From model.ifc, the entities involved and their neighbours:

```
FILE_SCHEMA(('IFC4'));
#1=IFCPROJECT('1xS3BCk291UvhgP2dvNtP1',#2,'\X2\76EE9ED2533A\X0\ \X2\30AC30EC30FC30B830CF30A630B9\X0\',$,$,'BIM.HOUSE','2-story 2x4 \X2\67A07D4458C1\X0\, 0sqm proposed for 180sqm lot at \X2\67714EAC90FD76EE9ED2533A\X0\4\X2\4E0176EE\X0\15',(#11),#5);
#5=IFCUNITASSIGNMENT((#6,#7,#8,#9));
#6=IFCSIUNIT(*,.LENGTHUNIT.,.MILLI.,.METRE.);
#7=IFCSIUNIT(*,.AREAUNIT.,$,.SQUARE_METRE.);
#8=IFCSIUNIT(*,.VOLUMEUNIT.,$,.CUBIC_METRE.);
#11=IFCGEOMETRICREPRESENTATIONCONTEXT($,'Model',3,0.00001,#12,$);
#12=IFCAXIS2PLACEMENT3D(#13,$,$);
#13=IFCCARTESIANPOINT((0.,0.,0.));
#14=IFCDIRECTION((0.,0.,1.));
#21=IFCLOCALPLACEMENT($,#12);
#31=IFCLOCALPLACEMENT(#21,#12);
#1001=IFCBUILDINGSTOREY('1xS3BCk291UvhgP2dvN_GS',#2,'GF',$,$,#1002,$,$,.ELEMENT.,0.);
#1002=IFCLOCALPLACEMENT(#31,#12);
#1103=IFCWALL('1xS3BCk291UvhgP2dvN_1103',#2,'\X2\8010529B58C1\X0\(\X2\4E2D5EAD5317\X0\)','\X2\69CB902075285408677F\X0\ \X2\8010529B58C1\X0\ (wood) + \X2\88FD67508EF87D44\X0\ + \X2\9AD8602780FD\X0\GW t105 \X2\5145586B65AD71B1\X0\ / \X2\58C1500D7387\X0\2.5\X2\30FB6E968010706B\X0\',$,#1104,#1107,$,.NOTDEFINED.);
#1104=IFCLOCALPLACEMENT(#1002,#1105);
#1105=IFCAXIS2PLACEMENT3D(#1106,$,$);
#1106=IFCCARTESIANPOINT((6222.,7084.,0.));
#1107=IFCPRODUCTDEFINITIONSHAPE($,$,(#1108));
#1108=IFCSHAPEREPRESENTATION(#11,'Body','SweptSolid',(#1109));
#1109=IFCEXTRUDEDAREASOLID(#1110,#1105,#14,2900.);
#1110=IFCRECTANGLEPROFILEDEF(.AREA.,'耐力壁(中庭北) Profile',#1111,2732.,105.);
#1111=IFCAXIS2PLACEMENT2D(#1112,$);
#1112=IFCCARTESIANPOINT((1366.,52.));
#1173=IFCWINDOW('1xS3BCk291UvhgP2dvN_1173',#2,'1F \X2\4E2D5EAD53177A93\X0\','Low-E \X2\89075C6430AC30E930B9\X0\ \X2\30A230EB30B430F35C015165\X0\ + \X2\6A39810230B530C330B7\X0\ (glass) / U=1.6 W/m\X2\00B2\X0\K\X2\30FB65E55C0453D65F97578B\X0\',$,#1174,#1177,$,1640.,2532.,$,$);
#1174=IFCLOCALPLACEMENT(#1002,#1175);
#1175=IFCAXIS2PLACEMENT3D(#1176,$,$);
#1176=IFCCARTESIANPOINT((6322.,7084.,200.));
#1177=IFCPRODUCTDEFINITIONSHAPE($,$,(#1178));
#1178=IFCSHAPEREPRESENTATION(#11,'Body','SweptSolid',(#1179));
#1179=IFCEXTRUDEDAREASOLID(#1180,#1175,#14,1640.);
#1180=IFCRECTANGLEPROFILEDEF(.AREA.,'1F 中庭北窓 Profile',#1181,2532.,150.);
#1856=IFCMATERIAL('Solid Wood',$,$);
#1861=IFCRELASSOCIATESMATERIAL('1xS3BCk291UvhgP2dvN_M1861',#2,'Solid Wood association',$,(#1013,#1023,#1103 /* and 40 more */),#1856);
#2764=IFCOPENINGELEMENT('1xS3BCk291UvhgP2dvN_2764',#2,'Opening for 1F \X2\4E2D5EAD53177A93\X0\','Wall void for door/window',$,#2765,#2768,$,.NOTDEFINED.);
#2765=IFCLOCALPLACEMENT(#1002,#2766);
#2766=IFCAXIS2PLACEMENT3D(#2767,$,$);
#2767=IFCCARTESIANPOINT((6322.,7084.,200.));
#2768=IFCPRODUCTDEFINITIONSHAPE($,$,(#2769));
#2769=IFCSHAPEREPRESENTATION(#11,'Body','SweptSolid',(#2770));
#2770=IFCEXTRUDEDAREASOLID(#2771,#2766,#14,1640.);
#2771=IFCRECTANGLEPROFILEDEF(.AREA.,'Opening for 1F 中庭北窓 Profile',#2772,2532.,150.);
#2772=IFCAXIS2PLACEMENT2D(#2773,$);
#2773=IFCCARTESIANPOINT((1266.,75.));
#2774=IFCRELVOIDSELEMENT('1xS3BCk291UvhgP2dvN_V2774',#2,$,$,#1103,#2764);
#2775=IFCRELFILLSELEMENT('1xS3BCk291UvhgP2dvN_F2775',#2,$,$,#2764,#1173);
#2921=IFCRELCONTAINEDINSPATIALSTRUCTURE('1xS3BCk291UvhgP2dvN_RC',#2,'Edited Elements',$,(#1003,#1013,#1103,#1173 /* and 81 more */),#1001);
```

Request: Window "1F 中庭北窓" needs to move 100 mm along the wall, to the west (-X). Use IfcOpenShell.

```python
import ifcopenshell
import ifcopenshell.api.geometry
import ifcopenshell.util.placement

model = ifcopenshell.open("model.ifc")

window = model.by_guid("1xS3BCk291UvhgP2dvN_1173")
opening = window.FillsVoids[0].RelatingOpeningElement
wall = opening.VoidsElements[0].RelatingBuildingElement

wall_matrix = ifcopenshell.util.placement.get_local_placement(wall.ObjectPlacement)
shift = wall_matrix[:3, 0] * -100.0
before = ifcopenshell.util.placement.get_local_placement(window.ObjectPlacement)[:3, 3].copy()

# The window is not placed relative to its opening, so move both.
for product in (opening, window):
    matrix = ifcopenshell.util.placement.get_local_placement(product.ObjectPlacement)
    matrix[:3, 3] += shift
    ifcopenshell.api.geometry.edit_object_placement(model, product=product, matrix=matrix, is_si=False)

after = ifcopenshell.util.placement.get_local_placement(window.ObjectPlacement)[:3, 3]
print("window moved by", (after - before).round(3) + 0.0)

model.write("model_updated.ifc")
```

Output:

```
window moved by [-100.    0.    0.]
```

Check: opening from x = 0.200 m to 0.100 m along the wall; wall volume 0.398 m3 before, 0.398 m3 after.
